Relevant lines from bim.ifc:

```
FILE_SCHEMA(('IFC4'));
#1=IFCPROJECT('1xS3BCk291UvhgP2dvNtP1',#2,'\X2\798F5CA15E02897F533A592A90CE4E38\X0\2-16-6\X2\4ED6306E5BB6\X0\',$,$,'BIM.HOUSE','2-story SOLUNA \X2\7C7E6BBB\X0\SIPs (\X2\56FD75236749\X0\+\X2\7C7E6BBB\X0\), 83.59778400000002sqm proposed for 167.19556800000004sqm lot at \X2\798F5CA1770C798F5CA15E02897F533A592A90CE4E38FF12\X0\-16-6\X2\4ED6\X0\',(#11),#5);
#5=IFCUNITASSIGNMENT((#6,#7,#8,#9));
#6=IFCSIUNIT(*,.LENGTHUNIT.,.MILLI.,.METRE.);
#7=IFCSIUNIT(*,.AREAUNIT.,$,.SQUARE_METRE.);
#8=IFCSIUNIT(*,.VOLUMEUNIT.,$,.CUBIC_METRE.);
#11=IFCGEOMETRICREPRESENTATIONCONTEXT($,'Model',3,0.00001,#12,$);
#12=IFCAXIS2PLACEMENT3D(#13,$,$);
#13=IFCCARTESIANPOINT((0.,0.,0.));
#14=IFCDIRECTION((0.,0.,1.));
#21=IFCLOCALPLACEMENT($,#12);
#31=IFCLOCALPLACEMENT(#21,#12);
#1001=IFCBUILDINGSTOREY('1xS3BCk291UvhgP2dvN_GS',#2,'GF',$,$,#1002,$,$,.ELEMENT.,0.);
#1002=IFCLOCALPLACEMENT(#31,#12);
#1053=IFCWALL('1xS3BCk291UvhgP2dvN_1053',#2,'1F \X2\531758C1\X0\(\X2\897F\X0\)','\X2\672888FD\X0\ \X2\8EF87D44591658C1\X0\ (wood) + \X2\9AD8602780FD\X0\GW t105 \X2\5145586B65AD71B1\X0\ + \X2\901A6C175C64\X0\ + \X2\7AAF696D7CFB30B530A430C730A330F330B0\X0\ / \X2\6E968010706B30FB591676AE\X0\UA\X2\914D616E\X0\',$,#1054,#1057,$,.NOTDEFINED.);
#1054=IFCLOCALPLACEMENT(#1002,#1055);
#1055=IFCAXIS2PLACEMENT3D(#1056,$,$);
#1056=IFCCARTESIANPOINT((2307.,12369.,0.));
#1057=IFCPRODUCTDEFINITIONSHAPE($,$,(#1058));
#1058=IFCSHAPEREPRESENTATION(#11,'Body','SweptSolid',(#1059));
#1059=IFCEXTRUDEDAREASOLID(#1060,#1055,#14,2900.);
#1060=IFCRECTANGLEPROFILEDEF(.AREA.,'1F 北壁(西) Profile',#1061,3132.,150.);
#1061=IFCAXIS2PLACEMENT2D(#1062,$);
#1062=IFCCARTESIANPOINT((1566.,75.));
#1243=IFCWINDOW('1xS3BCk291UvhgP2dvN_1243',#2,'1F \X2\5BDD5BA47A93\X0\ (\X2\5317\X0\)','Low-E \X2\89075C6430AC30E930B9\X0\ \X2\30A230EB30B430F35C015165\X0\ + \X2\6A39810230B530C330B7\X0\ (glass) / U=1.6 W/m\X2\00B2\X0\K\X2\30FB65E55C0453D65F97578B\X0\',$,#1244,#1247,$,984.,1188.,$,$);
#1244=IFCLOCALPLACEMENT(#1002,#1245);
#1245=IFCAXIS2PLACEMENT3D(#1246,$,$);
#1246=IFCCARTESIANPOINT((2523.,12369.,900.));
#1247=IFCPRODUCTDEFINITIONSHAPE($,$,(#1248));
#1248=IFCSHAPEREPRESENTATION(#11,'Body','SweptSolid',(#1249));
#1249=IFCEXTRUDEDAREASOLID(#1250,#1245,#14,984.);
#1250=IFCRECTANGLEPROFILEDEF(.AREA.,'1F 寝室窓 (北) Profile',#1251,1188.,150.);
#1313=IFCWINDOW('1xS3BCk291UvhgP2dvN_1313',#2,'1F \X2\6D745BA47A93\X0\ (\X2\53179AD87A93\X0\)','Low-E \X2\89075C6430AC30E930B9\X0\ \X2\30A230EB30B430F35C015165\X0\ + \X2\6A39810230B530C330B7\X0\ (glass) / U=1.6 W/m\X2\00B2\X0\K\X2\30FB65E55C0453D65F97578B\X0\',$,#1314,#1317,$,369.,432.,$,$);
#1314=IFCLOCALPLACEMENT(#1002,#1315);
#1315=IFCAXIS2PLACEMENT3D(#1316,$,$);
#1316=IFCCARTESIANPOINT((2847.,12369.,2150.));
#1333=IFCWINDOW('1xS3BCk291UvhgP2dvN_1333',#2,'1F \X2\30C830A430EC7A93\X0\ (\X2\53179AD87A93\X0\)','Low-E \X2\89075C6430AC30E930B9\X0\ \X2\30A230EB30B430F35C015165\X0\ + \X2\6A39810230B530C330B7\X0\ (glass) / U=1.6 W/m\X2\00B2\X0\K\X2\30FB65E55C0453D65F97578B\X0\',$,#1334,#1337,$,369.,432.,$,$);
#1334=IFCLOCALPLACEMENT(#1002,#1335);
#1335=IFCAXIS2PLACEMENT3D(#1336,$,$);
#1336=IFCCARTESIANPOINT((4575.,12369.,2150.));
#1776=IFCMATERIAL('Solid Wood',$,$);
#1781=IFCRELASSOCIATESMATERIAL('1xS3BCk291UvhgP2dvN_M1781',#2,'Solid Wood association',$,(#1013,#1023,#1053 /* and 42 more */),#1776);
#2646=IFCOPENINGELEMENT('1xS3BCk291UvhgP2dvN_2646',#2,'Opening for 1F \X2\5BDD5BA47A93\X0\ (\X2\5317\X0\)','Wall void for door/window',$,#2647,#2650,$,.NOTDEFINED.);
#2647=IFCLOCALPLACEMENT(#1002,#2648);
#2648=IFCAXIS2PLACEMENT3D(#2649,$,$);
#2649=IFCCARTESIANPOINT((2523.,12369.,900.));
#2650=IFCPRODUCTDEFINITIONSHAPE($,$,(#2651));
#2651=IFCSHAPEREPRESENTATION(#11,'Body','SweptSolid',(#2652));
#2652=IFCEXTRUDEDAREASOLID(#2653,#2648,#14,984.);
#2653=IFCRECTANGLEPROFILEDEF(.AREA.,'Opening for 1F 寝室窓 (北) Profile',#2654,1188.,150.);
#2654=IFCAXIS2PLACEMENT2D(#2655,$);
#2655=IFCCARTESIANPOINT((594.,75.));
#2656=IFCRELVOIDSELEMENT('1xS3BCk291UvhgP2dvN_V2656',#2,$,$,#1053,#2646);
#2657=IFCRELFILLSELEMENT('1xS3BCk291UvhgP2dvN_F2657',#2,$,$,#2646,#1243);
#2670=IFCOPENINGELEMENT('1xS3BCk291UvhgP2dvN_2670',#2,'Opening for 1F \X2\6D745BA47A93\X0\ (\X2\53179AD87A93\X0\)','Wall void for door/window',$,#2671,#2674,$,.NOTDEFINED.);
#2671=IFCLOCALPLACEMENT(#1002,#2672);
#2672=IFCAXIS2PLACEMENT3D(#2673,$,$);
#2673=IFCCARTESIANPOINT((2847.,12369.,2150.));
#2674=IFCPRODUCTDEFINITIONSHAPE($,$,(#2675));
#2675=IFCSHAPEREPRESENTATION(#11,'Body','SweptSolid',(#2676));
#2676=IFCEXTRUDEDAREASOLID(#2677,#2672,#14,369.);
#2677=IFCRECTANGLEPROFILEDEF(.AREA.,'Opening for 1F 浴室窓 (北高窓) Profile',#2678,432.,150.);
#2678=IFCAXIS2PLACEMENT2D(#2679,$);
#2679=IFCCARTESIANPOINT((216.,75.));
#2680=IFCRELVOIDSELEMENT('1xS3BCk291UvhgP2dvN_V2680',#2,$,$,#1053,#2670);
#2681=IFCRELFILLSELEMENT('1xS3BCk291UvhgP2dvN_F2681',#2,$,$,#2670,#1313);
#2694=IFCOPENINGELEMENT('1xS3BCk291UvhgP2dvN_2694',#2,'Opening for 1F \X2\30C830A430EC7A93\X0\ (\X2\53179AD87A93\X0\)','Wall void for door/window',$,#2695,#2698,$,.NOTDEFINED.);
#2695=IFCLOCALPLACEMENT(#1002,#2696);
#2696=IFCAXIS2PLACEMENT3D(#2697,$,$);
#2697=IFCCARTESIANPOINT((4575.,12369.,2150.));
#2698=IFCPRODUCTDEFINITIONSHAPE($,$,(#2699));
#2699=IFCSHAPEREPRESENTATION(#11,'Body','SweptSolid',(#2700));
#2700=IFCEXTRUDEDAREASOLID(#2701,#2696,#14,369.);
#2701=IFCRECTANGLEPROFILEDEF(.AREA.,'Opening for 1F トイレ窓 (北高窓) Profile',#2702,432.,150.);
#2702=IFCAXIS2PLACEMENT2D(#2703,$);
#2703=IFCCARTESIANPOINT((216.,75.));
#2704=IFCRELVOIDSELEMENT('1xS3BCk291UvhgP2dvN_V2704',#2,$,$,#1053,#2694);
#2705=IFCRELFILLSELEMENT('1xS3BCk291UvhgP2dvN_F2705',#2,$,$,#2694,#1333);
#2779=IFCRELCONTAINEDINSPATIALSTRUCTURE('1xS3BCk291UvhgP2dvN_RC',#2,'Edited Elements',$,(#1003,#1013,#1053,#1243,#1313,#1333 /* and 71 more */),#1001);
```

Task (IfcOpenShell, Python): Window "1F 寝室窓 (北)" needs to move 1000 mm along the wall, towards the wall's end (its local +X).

```python
import ifcopenshell
import ifcopenshell.api.geometry
import ifcopenshell.util.placement
import ifcopenshell.util.unit

model = ifcopenshell.open("bim.ifc")
unit_scale = ifcopenshell.util.unit.calculate_unit_scale(model)

window = model.by_guid("1xS3BCk291UvhgP2dvN_1243")
opening = window.FillsVoids[0].RelatingOpeningElement
wall = opening.VoidsElements[0].RelatingBuildingElement

wall_matrix = ifcopenshell.util.placement.get_local_placement(wall.ObjectPlacement)
shift = wall_matrix[:3, 0] * 1 / unit_scale
before = ifcopenshell.util.placement.get_local_placement(window.ObjectPlacement)[:3, 3].copy()

# The window is not placed relative to its opening, so move both.
for product in (opening, window):
    matrix = ifcopenshell.util.placement.get_local_placement(product.ObjectPlacement)
    matrix[:3, 3] += shift
    ifcopenshell.api.geometry.edit_object_placement(model, product=product, matrix=matrix, is_si=False)

after = ifcopenshell.util.placement.get_local_placement(window.ObjectPlacement)[:3, 3]
print("window moved by", (after - before).round(3) + 0.0)

model.write("bim_v2.ifc")
```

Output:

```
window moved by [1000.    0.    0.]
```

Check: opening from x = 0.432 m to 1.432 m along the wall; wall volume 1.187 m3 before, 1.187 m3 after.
